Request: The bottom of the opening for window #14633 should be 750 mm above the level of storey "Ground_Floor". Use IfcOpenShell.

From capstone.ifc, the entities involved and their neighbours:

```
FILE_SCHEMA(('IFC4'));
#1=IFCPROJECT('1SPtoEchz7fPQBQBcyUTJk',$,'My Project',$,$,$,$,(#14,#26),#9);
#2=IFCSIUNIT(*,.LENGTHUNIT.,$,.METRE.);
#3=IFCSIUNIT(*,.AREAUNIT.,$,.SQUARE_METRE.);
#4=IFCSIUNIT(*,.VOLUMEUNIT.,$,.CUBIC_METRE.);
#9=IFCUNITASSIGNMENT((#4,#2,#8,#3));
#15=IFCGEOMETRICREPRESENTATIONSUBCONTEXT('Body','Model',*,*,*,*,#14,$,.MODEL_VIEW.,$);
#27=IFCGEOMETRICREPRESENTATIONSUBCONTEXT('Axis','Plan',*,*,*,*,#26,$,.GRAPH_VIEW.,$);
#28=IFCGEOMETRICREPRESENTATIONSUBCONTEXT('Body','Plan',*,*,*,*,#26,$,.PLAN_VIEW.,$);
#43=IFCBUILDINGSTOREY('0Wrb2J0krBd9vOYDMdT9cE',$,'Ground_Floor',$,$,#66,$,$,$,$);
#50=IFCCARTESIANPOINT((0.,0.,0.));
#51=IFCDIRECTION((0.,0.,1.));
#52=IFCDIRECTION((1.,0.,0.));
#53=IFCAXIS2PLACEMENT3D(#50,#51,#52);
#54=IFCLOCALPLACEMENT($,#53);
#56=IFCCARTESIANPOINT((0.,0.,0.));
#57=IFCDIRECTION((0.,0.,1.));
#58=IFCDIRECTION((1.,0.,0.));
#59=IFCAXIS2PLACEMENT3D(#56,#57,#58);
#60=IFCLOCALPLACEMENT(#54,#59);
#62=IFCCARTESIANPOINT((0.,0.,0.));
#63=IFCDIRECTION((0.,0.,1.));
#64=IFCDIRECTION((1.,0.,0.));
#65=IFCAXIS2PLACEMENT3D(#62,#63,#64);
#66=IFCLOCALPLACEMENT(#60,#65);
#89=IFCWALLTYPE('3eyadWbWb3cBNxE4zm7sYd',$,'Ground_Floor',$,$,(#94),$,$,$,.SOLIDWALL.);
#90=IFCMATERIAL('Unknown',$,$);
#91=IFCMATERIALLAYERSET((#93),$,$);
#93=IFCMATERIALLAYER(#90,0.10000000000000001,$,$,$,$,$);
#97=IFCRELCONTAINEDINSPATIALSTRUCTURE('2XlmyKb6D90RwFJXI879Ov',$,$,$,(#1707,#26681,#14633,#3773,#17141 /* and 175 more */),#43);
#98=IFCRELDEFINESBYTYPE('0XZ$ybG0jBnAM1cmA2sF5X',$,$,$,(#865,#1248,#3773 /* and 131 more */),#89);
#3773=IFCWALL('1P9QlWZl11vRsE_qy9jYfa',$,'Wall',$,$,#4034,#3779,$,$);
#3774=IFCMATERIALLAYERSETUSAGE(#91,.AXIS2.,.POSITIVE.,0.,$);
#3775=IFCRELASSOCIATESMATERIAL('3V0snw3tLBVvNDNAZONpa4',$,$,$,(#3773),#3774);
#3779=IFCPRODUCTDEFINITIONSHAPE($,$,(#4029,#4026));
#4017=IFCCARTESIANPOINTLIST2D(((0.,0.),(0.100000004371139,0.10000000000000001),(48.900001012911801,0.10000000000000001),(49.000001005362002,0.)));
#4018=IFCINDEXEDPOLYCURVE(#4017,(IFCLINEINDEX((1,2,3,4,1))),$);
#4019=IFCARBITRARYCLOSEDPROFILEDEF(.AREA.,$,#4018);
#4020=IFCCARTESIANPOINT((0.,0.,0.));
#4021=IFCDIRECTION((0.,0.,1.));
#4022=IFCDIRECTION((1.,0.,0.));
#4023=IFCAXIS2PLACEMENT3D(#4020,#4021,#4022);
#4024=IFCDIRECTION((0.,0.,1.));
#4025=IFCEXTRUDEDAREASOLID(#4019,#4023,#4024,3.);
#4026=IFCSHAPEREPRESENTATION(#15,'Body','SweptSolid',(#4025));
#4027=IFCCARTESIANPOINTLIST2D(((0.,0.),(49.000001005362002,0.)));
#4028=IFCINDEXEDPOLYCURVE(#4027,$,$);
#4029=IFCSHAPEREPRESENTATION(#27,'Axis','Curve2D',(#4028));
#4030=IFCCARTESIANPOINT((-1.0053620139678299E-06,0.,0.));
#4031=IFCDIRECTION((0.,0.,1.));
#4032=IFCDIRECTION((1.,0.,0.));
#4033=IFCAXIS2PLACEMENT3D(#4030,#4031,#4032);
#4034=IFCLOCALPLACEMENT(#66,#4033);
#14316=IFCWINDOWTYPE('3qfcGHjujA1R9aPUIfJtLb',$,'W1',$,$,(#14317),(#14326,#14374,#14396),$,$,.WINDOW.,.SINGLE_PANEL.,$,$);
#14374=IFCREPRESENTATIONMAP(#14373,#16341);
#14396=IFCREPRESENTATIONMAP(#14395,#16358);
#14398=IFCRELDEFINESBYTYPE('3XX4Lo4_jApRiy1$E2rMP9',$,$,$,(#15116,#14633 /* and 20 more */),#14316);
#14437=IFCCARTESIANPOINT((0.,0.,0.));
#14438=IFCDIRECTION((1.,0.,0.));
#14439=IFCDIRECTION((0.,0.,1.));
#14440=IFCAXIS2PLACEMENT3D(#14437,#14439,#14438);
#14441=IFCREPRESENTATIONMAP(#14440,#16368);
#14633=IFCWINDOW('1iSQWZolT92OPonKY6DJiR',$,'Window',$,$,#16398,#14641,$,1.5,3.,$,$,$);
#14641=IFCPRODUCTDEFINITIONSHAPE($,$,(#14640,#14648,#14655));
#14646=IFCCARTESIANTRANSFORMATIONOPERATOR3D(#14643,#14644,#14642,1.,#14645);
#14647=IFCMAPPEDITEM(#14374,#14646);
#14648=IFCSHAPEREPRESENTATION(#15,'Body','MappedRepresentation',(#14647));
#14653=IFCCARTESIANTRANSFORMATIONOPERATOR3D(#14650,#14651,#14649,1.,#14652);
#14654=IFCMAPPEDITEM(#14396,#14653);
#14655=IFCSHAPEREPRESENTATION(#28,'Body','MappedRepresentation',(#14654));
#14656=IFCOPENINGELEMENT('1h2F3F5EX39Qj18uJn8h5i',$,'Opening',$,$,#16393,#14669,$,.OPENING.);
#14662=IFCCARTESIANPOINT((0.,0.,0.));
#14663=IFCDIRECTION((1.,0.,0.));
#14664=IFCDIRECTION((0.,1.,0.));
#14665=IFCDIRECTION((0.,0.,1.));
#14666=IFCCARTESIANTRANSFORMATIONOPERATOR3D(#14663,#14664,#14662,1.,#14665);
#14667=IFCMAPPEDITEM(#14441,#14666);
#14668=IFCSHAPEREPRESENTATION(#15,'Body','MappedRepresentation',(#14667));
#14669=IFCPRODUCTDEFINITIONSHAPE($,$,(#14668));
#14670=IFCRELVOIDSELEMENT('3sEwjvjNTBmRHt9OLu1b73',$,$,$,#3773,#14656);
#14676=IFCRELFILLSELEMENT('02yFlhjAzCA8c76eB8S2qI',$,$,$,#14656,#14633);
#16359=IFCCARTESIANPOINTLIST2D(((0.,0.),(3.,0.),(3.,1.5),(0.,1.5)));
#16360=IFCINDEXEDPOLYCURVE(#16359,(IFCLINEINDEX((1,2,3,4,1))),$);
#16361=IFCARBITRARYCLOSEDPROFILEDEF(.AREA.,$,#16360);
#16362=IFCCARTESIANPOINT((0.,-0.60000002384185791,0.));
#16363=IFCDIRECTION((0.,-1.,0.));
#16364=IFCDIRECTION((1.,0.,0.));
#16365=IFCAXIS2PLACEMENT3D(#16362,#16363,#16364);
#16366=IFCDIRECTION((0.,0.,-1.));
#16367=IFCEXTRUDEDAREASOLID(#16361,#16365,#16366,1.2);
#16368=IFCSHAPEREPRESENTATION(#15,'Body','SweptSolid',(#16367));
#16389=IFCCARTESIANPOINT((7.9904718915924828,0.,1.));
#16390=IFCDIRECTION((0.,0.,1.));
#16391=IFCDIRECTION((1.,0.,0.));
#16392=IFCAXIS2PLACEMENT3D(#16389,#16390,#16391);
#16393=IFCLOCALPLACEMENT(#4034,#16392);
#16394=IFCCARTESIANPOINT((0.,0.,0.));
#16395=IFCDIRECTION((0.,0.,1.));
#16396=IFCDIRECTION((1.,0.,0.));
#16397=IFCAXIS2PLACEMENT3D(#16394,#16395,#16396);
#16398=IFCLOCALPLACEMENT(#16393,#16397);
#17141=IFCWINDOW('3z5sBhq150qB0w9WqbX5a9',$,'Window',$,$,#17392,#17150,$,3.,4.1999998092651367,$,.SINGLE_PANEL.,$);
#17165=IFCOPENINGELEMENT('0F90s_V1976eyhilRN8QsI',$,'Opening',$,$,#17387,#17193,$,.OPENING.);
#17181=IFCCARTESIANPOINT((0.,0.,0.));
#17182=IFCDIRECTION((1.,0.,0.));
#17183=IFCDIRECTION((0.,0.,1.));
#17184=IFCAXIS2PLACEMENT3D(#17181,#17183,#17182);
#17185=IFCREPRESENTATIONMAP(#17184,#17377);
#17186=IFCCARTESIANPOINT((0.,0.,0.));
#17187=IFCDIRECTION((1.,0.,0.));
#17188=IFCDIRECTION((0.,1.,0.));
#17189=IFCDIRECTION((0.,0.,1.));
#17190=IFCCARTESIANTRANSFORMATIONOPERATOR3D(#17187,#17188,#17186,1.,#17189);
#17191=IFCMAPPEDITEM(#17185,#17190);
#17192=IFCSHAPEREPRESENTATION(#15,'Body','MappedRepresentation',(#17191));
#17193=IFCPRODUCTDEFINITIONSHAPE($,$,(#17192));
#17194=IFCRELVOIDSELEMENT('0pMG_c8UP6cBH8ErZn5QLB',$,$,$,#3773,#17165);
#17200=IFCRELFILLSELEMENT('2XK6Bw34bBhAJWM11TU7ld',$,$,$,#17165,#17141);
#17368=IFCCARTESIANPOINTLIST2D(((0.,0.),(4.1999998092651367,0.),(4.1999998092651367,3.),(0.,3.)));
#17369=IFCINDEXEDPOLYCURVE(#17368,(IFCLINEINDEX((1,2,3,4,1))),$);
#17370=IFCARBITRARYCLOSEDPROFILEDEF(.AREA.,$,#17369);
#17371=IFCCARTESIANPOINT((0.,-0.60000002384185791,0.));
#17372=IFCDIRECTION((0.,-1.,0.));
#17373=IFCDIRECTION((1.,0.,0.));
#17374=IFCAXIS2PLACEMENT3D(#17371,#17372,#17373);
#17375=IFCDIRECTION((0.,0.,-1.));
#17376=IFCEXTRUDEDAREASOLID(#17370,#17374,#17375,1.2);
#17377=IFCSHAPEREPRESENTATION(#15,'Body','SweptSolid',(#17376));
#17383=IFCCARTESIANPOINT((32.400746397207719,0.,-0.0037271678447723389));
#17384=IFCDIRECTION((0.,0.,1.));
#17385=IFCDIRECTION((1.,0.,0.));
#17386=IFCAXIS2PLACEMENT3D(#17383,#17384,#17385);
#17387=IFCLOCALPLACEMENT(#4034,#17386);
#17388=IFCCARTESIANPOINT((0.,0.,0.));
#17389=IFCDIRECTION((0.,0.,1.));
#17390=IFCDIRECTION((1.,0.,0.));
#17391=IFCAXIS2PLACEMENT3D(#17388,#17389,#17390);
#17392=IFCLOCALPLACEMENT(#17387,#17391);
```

```python
import numpy as np
import ifcopenshell
import ifcopenshell.api.geometry
import ifcopenshell.geom
import ifcopenshell.util.element
import ifcopenshell.util.placement
import ifcopenshell.util.shape
import ifcopenshell.util.unit

model = ifcopenshell.open("capstone.ifc")
unit_scale = ifcopenshell.util.unit.calculate_unit_scale(model)

window = model.by_guid("1iSQWZolT92OPonKY6DJiR")
opening = window.FillsVoids[0].RelatingOpeningElement
storey = ifcopenshell.util.element.get_container(window, ifc_class="IfcBuildingStorey")
level = ifcopenshell.util.placement.get_local_placement(storey.ObjectPlacement)[2, 3]

# The opening's origin need not be at the sill, so measure its lowest point.
shape = ifcopenshell.geom.create_shape(ifcopenshell.geom.settings(), opening)
bottom = ifcopenshell.util.shape.get_shape_bottom_elevation(shape, shape.geometry) / unit_scale
dz = level + 0.75 - bottom

shift = np.array([0.0, 0.0, dz])
# The window is placed relative to its opening, so it follows when the opening moves.
matrix = ifcopenshell.util.placement.get_local_placement(opening.ObjectPlacement)
matrix[:3, 3] += shift
ifcopenshell.api.geometry.edit_object_placement(
    model, product=opening, matrix=matrix, is_si=False, should_transform_children=True
)

print(f"moved by {dz * unit_scale:+.3f} m")

model.write("capstone_rev.ifc")
```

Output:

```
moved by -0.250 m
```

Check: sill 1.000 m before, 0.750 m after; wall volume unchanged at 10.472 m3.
